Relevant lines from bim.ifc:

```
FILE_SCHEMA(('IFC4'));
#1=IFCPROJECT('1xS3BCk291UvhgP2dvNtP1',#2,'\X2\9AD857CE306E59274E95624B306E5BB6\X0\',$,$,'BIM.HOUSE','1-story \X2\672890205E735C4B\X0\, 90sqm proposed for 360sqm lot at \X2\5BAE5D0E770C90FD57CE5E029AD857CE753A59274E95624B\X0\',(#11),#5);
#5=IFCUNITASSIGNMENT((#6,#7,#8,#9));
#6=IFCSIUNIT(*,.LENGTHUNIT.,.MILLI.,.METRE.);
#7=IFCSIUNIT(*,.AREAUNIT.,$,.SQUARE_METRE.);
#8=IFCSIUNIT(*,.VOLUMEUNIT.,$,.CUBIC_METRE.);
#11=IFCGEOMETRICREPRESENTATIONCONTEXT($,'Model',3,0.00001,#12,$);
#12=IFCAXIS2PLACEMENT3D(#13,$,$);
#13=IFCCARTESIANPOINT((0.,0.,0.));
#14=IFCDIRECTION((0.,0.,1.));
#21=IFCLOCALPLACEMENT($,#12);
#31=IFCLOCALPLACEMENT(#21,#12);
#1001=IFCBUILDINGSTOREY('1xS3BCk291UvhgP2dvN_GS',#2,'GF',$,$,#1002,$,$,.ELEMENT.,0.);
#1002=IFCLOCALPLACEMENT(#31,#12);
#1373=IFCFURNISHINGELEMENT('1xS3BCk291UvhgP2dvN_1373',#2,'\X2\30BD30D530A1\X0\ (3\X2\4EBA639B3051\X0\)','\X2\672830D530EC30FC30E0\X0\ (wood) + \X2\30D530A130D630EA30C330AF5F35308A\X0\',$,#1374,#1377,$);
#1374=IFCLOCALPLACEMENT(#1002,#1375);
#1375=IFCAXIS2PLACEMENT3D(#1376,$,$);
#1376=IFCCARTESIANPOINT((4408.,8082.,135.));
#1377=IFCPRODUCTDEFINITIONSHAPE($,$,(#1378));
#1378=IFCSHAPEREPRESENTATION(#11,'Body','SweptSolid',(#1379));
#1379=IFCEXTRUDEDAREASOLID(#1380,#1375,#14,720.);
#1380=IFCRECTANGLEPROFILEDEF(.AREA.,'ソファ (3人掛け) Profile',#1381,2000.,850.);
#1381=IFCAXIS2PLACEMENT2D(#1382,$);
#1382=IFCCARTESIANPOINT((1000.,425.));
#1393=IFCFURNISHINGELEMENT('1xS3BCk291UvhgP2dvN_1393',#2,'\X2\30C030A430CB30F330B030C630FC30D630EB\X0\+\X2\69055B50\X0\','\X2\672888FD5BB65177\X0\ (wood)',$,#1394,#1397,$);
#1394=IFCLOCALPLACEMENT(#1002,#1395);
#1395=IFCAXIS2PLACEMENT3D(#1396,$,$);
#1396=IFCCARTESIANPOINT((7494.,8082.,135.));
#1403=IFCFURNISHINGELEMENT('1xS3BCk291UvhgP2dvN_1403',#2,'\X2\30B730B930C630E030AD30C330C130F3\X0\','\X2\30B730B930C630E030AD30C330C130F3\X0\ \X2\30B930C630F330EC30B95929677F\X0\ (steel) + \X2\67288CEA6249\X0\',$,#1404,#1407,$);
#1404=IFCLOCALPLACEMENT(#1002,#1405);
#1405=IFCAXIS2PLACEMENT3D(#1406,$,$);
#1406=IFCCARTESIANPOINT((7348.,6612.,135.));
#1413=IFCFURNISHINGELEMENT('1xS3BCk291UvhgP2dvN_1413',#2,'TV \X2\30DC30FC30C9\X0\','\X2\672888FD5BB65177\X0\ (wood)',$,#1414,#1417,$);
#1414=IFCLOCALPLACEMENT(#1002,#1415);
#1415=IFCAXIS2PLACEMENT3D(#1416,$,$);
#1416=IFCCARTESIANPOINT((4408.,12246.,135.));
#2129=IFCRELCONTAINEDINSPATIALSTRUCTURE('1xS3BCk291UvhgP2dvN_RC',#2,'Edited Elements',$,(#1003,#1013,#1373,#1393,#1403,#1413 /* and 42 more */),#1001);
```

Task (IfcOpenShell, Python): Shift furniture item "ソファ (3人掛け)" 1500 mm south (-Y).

```python
import ifcopenshell
import ifcopenshell.api.geometry
import ifcopenshell.util.placement
import ifcopenshell.util.unit

model = ifcopenshell.open("bim.ifc")
unit_scale = ifcopenshell.util.unit.calculate_unit_scale(model)

item = model.by_guid("1xS3BCk291UvhgP2dvN_1373")
matrix = ifcopenshell.util.placement.get_local_placement(item.ObjectPlacement)
matrix[1, 3] -= 1.5 / unit_scale
ifcopenshell.api.geometry.edit_object_placement(model, product=item, matrix=matrix, is_si=False)

print(ifcopenshell.util.placement.get_local_placement(item.ObjectPlacement).round(3) + 0.0)

model.write("bim-out.ifc")
```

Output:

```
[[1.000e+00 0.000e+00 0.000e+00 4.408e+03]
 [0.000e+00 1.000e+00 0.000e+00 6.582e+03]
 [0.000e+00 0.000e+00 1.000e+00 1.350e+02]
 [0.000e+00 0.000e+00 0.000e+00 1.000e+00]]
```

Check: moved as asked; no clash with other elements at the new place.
